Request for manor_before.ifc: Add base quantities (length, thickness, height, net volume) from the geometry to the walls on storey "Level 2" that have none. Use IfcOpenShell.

First a look at what the model holds.

```python
import ifcopenshell
import ifcopenshell.util.element
import ifcopenshell.util.unit

model = ifcopenshell.open("manor_before.ifc")
print(model.schema)
for unit_type in ("LENGTHUNIT", "AREAUNIT", "VOLUMEUNIT"):
    print(unit_type, ifcopenshell.util.unit.calculate_unit_scale(model, unit_type))
storey = next(s for s in model.by_type("IfcBuildingStorey") if s.Name == "Level 2")
walls = [e for e in ifcopenshell.util.element.get_decomposition(storey) if e.is_a("IfcWall")]
for e in sorted(walls, key=lambda e: e.id()):
    print(e.id(), e.is_a(), e.Name, list(ifcopenshell.util.element.get_psets(e, qtos_only=True)), sep=" | ")
```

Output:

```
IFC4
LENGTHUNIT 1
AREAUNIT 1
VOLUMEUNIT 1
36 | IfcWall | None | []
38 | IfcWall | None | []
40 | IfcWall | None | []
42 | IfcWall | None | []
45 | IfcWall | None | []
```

```python
import ifcopenshell
import ifcopenshell.api.pset
import ifcopenshell.geom
import ifcopenshell.util.element
import ifcopenshell.util.shape
import ifcopenshell.util.unit

model = ifcopenshell.open("manor_before.ifc")
unit_scale = ifcopenshell.util.unit.calculate_unit_scale(model)
volume_scale = ifcopenshell.util.unit.calculate_unit_scale(model, "VOLUMEUNIT")
settings = ifcopenshell.geom.settings()

storey = next(s for s in model.by_type("IfcBuildingStorey") if s.Name == "Level 2")
walls = [e for e in ifcopenshell.util.element.get_decomposition(storey) if e.is_a("IfcWall")]

for e in sorted(walls, key=lambda e: e.id()):
    if ifcopenshell.util.element.get_psets(e, qtos_only=True, should_inherit=False):
        continue
    # Geometry comes back in metres, in the element's own axes.
    shape = ifcopenshell.geom.create_shape(settings, e)
    values = {
        "Length": ifcopenshell.util.shape.get_x(shape.geometry) / unit_scale,
        "Width": ifcopenshell.util.shape.get_y(shape.geometry) / unit_scale,
        "Height": ifcopenshell.util.shape.get_z(shape.geometry) / unit_scale,
        "NetVolume": ifcopenshell.util.shape.get_volume(shape.geometry) / volume_scale,
    }
    qto = ifcopenshell.api.pset.add_qto(model, product=e, name="Qto_WallBaseQuantities")
    ifcopenshell.api.pset.edit_qto(model, qto=qto, properties=values)
    print(e.id(), {k: round(v, 3) for k, v in values.items()})

model.write("manor_before_v2.ifc")
```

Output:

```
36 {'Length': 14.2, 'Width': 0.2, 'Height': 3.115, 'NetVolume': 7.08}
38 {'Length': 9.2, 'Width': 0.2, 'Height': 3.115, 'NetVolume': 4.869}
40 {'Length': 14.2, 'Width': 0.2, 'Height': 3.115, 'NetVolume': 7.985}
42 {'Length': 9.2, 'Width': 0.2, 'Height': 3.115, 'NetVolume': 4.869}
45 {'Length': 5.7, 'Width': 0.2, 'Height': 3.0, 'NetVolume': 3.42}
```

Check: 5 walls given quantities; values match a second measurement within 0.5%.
